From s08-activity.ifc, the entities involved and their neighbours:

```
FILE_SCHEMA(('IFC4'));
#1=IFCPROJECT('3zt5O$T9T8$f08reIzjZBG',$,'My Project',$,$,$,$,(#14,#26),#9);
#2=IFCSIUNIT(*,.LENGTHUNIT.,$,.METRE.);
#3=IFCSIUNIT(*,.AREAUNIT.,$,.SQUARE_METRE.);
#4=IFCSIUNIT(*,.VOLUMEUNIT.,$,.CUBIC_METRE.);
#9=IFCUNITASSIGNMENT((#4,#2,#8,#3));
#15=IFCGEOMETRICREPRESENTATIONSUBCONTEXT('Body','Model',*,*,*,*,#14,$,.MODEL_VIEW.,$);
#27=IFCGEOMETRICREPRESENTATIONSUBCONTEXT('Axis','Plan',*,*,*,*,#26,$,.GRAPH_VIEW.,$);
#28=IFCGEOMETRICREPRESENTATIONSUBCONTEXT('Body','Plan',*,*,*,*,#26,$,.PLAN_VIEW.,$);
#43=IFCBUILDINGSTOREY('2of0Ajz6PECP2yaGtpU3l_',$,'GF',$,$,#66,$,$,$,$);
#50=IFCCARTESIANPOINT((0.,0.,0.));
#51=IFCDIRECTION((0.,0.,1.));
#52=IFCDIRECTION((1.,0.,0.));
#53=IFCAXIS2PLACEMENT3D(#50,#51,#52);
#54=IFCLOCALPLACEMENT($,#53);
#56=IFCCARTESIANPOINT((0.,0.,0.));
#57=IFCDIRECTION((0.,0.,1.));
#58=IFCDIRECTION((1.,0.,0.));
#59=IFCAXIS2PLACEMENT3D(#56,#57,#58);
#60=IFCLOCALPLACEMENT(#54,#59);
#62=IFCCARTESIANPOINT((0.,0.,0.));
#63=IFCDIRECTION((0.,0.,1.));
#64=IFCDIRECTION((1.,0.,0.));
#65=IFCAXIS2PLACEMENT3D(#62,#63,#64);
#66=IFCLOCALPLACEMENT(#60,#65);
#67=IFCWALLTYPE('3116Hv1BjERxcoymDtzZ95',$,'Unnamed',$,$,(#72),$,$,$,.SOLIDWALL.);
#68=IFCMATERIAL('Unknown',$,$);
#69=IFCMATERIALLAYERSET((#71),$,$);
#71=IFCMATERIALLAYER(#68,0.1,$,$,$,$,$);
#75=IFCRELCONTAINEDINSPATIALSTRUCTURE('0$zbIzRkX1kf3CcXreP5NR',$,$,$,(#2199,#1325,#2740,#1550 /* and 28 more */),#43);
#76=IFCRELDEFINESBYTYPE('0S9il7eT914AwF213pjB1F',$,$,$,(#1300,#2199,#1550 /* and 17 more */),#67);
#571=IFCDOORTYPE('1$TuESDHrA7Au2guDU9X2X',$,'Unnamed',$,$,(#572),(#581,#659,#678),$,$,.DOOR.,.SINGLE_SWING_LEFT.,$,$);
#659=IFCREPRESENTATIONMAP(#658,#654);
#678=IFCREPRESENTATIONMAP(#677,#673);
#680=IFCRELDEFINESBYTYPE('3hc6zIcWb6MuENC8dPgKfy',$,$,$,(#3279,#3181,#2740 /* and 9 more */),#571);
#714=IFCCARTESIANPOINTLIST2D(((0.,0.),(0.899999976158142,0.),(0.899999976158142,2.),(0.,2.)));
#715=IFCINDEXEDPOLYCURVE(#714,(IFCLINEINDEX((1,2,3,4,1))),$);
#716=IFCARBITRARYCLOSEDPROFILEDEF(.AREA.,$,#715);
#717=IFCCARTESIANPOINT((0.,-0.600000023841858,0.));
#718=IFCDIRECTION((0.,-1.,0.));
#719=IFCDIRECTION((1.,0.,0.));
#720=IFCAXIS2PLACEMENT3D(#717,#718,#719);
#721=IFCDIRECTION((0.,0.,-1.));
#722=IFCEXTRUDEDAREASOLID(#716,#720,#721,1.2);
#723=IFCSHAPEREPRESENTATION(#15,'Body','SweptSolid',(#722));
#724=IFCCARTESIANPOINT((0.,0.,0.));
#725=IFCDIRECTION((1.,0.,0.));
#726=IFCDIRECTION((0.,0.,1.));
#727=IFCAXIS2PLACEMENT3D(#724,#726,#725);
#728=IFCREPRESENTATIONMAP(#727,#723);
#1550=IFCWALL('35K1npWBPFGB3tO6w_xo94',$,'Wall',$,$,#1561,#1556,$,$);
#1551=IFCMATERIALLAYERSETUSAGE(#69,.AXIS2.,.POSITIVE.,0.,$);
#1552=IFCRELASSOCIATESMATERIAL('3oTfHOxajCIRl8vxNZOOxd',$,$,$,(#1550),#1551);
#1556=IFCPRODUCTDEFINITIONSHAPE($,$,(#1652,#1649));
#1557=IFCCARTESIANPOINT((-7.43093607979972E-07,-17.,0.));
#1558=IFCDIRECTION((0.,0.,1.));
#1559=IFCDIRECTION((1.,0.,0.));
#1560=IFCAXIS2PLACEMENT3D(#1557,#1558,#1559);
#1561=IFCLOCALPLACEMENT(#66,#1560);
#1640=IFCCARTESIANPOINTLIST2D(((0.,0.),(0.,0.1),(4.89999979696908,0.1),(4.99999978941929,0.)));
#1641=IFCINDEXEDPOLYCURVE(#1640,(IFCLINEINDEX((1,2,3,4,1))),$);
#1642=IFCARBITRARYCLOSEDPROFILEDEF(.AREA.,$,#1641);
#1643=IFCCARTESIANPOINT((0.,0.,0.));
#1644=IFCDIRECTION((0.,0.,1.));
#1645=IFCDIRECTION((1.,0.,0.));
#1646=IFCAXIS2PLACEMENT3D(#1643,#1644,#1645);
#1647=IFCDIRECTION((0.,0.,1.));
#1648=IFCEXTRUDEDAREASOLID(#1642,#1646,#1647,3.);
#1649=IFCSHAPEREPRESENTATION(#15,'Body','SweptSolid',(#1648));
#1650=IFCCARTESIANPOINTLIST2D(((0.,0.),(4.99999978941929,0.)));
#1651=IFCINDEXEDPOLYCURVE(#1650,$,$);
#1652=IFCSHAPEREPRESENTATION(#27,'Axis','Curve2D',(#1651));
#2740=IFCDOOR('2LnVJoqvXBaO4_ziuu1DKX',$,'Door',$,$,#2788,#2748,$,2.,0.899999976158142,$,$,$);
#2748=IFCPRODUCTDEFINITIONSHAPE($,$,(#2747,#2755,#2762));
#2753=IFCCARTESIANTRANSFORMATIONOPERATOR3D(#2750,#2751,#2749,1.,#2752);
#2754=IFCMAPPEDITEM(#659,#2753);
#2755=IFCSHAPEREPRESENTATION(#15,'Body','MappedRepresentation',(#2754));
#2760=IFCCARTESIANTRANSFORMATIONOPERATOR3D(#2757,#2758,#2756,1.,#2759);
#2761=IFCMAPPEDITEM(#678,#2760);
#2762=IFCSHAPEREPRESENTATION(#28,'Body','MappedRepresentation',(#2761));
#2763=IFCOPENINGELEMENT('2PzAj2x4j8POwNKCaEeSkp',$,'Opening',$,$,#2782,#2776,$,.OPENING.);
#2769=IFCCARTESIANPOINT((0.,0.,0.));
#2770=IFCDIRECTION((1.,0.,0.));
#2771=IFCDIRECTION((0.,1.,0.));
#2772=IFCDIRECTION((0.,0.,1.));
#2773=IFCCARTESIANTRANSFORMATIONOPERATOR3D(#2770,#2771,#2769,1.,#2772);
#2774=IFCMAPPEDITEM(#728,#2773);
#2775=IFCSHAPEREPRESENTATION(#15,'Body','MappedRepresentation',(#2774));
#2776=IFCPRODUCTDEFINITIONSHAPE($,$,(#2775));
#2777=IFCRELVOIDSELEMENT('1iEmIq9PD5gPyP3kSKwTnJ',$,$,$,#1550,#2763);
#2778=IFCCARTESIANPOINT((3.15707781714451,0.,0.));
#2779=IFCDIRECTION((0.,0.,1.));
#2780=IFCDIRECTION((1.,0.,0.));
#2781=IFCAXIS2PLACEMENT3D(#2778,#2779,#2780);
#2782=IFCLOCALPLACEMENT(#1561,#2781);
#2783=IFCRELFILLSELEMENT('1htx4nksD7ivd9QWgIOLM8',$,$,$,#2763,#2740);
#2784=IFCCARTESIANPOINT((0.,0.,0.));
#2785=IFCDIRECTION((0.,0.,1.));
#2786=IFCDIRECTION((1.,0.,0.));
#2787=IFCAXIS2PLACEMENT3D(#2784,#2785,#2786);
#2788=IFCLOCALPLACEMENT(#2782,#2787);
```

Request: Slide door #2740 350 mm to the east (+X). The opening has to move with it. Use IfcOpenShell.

```python
import ifcopenshell
import ifcopenshell.api.geometry
import ifcopenshell.util.placement
import ifcopenshell.util.unit

model = ifcopenshell.open("s08-activity.ifc")
unit_scale = ifcopenshell.util.unit.calculate_unit_scale(model)

door = model.by_guid("2LnVJoqvXBaO4_ziuu1DKX")
opening = door.FillsVoids[0].RelatingOpeningElement
wall = opening.VoidsElements[0].RelatingBuildingElement

wall_matrix = ifcopenshell.util.placement.get_local_placement(wall.ObjectPlacement)
shift = wall_matrix[:3, 0] * 0.35 / unit_scale
before = ifcopenshell.util.placement.get_local_placement(door.ObjectPlacement)[:3, 3].copy()

# The door is placed relative to its opening, so it follows when the opening moves.
matrix = ifcopenshell.util.placement.get_local_placement(opening.ObjectPlacement)
matrix[:3, 3] += shift
ifcopenshell.api.geometry.edit_object_placement(
    model, product=opening, matrix=matrix, is_si=False, should_transform_children=True
)

after = ifcopenshell.util.placement.get_local_placement(door.ObjectPlacement)[:3, 3]
print("door moved by", (after - before).round(3) + 0.0)

model.write("s08-activity_edited.ifc")
```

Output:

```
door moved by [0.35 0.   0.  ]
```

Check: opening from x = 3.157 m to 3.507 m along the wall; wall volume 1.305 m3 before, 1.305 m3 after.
